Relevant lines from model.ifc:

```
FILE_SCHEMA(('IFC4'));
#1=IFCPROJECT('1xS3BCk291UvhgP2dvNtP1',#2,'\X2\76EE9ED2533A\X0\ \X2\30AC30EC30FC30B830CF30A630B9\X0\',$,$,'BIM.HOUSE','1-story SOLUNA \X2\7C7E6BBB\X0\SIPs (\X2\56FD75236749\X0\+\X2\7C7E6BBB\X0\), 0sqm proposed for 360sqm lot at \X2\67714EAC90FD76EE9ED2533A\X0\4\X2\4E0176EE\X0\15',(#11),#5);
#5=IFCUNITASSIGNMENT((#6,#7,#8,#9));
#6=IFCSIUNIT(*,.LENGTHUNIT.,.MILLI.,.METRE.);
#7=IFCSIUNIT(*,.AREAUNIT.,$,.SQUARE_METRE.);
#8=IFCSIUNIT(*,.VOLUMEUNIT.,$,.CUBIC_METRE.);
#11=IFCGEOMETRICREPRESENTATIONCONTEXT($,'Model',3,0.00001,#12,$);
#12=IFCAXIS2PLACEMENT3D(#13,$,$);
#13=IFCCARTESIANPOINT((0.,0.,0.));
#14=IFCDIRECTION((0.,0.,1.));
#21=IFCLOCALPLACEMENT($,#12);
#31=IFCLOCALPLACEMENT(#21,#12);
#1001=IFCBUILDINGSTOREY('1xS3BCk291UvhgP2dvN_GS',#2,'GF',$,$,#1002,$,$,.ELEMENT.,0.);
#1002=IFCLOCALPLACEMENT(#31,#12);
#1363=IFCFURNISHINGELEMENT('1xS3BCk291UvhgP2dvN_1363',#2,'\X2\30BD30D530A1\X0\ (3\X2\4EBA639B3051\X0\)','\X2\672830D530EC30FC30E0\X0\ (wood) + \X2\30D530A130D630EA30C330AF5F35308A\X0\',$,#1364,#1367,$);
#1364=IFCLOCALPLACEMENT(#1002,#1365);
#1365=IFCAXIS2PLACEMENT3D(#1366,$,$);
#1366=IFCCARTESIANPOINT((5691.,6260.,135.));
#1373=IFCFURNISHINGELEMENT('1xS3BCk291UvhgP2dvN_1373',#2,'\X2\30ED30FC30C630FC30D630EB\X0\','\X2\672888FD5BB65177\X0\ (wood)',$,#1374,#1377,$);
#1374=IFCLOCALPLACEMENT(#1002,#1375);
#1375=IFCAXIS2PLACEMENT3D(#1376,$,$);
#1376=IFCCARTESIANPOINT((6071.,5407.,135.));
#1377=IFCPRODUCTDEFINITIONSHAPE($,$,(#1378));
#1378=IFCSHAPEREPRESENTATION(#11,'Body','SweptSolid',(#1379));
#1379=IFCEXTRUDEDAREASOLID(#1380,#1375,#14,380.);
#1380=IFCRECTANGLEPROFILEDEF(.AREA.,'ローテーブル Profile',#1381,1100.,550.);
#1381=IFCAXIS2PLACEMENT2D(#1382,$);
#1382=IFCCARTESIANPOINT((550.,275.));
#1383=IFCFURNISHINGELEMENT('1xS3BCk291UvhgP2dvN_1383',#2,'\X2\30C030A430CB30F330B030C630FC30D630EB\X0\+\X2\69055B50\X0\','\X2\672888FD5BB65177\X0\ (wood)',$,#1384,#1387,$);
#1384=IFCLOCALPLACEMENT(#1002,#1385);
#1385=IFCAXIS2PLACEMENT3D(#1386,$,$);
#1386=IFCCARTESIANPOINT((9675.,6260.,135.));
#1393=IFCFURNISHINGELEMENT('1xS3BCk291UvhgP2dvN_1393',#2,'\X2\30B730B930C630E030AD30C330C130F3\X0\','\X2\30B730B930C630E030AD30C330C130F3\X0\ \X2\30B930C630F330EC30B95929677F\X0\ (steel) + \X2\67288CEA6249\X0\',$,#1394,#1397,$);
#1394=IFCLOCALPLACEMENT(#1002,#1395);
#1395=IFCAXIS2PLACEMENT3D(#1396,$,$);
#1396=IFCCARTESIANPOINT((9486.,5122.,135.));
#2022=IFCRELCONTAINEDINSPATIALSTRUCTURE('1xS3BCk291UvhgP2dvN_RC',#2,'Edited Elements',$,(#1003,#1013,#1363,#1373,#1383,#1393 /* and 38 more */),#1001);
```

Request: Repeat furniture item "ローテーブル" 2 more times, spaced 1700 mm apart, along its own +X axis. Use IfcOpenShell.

```python
import ifcopenshell
import ifcopenshell.api.geometry
import ifcopenshell.api.root
import ifcopenshell.util.element
import ifcopenshell.util.placement
import ifcopenshell.util.unit

model = ifcopenshell.open("model.ifc")
unit_scale = ifcopenshell.util.unit.calculate_unit_scale(model)


def reuse_history(source, copy):
    """copy_class also copies each property set's owner history, people and application; keep the originals."""
    for rel in copy.IsDefinedBy:
        if rel.is_a("IfcRelDefinesByProperties") and (history := rel.RelatingPropertyDefinition.OwnerHistory):
            rel.RelatingPropertyDefinition.OwnerHistory = source.OwnerHistory
            ifcopenshell.util.element.remove_deep2(model, history)


source = model.by_guid("1xS3BCk291UvhgP2dvN_1373")
base = ifcopenshell.util.placement.get_local_placement(source.ObjectPlacement)
step = base[:3, 0] * 1.7 / unit_scale

for i in range(1, 3):
    copy = ifcopenshell.api.root.copy_class(model, product=source)
    copy.Representation = ifcopenshell.util.element.copy_deep(
        model, source.Representation, exclude=["IfcGeometricRepresentationContext", "IfcRepresentationMap"]
    )
    reuse_history(source, copy)
    matrix = base.copy()
    matrix[:3, 3] += i * step
    print("added at", matrix[:3, 3].round(3) + 0.0)
    ifcopenshell.api.geometry.edit_object_placement(model, product=copy, matrix=matrix, is_si=False)

model.write("model_edited.ifc")
```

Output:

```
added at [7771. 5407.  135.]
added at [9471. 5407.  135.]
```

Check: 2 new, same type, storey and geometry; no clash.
